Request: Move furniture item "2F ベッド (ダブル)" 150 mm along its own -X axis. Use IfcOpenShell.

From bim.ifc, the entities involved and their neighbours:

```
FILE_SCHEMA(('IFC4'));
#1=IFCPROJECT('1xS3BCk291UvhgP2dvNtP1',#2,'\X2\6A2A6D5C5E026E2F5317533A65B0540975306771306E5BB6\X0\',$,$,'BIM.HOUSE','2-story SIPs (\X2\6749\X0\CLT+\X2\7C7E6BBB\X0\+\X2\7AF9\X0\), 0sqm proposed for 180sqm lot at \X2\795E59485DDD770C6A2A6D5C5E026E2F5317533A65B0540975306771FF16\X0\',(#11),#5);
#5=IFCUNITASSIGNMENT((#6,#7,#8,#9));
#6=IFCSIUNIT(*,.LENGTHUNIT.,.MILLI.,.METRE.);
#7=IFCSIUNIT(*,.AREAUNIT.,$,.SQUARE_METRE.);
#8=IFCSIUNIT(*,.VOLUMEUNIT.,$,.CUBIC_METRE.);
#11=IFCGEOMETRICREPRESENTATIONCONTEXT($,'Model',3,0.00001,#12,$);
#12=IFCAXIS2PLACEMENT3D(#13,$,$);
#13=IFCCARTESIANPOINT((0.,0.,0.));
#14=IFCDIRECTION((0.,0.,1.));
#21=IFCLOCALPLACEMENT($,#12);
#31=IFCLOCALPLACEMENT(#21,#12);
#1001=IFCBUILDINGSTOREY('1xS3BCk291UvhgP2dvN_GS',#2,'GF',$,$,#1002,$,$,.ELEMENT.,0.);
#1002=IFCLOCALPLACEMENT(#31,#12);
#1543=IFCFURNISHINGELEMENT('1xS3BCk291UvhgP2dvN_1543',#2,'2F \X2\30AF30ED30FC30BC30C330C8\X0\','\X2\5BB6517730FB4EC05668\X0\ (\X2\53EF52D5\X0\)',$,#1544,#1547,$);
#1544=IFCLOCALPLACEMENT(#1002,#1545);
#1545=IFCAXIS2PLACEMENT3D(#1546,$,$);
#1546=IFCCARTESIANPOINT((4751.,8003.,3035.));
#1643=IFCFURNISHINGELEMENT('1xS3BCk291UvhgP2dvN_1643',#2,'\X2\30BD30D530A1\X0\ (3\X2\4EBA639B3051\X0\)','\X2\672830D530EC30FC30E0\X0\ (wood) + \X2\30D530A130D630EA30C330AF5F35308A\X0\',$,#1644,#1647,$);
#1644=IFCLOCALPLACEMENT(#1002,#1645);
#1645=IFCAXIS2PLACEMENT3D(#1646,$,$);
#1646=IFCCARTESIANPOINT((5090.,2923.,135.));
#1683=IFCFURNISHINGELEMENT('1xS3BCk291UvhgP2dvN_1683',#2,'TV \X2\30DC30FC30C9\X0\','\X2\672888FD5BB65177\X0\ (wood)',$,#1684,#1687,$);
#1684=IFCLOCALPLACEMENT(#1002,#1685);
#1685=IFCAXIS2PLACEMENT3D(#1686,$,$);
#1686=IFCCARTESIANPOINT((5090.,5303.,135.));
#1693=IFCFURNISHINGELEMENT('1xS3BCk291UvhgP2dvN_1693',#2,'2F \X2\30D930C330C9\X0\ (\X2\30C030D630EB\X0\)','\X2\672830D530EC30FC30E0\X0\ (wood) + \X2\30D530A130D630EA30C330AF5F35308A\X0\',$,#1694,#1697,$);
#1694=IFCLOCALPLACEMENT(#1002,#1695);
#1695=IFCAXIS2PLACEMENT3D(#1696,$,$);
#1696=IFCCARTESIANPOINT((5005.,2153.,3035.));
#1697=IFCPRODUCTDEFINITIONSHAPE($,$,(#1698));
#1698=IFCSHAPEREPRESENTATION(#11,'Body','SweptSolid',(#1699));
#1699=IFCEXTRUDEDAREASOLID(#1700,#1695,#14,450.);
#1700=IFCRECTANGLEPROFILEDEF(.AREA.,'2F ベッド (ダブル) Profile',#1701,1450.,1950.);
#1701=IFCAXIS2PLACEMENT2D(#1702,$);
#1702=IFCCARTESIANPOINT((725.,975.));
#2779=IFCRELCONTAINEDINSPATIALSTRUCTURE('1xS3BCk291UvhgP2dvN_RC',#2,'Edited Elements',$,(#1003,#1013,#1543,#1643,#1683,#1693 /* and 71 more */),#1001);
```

```python
import ifcopenshell
import ifcopenshell.api.geometry
import ifcopenshell.util.placement
import ifcopenshell.util.unit

model = ifcopenshell.open("bim.ifc")
unit_scale = ifcopenshell.util.unit.calculate_unit_scale(model)

item = model.by_guid("1xS3BCk291UvhgP2dvN_1693")
matrix = ifcopenshell.util.placement.get_local_placement(item.ObjectPlacement)
matrix[:3, 3] -= matrix[:3, 0] * 0.15 / unit_scale
ifcopenshell.api.geometry.edit_object_placement(model, product=item, matrix=matrix, is_si=False)

print(ifcopenshell.util.placement.get_local_placement(item.ObjectPlacement).round(3) + 0.0)

model.write("bim_v2.ifc")
```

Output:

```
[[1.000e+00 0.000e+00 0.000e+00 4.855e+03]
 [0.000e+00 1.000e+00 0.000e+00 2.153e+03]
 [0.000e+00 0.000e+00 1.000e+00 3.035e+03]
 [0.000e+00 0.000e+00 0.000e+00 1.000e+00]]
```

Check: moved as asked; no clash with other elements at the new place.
